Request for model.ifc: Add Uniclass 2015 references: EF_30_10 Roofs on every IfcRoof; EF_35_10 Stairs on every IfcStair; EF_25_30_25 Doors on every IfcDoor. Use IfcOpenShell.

First a look at what the model holds.

```python
import ifcopenshell

model = ifcopenshell.open("model.ifc")
print(model.schema)
print("classifications:", [c.Name for c in model.by_type("IfcClassification")])
for ifc_class in ("IfcDoor", "IfcRoof", "IfcStair", "IfcWall", "IfcWindow"):
    print(ifc_class, len(model.by_type(ifc_class)))
```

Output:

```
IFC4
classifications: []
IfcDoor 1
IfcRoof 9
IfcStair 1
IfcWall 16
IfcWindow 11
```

```python
import ifcopenshell
import ifcopenshell.api.classification

model = ifcopenshell.open("model.ifc")

system = ifcopenshell.api.classification.add_classification(model, classification="Uniclass 2015")

codes = {
    "IfcRoof": ("EF_30_10", "Roofs"),
    "IfcStair": ("EF_35_10", "Stairs"),
    "IfcDoor": ("EF_25_30_25", "Doors"),
}
for ifc_class, (code, name) in codes.items():
    products = model.by_type(ifc_class)
    ifcopenshell.api.classification.add_reference(
        model, products=products, classification=system, identification=code, name=name
    )
    print(code, len(products))

model.write("model_v2.ifc")
```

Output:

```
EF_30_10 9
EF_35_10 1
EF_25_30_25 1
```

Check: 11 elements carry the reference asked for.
